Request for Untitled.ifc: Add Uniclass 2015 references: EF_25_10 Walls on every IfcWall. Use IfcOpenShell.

First a look at what the model holds.

```python
import ifcopenshell

model = ifcopenshell.open("Untitled.ifc")
print(model.schema)
print("classifications:", [c.Name for c in model.by_type("IfcClassification")])
for ifc_class in ("IfcDoor", "IfcRoof", "IfcStair", "IfcWall", "IfcWindow"):
    print(ifc_class, len(model.by_type(ifc_class)))
```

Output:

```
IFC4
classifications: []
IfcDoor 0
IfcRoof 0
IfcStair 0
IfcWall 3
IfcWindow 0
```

```python
import ifcopenshell
import ifcopenshell.api.classification

model = ifcopenshell.open("Untitled.ifc")

system = ifcopenshell.api.classification.add_classification(model, classification="Uniclass 2015")

codes = {
    "IfcWall": ("EF_25_10", "Walls"),
}
for ifc_class, (code, name) in codes.items():
    products = model.by_type(ifc_class)
    ifcopenshell.api.classification.add_reference(
        model, products=products, classification=system, identification=code, name=name
    )
    print(code, len(products))

model.write("Untitled-out.ifc")
```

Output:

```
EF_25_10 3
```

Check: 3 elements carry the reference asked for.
